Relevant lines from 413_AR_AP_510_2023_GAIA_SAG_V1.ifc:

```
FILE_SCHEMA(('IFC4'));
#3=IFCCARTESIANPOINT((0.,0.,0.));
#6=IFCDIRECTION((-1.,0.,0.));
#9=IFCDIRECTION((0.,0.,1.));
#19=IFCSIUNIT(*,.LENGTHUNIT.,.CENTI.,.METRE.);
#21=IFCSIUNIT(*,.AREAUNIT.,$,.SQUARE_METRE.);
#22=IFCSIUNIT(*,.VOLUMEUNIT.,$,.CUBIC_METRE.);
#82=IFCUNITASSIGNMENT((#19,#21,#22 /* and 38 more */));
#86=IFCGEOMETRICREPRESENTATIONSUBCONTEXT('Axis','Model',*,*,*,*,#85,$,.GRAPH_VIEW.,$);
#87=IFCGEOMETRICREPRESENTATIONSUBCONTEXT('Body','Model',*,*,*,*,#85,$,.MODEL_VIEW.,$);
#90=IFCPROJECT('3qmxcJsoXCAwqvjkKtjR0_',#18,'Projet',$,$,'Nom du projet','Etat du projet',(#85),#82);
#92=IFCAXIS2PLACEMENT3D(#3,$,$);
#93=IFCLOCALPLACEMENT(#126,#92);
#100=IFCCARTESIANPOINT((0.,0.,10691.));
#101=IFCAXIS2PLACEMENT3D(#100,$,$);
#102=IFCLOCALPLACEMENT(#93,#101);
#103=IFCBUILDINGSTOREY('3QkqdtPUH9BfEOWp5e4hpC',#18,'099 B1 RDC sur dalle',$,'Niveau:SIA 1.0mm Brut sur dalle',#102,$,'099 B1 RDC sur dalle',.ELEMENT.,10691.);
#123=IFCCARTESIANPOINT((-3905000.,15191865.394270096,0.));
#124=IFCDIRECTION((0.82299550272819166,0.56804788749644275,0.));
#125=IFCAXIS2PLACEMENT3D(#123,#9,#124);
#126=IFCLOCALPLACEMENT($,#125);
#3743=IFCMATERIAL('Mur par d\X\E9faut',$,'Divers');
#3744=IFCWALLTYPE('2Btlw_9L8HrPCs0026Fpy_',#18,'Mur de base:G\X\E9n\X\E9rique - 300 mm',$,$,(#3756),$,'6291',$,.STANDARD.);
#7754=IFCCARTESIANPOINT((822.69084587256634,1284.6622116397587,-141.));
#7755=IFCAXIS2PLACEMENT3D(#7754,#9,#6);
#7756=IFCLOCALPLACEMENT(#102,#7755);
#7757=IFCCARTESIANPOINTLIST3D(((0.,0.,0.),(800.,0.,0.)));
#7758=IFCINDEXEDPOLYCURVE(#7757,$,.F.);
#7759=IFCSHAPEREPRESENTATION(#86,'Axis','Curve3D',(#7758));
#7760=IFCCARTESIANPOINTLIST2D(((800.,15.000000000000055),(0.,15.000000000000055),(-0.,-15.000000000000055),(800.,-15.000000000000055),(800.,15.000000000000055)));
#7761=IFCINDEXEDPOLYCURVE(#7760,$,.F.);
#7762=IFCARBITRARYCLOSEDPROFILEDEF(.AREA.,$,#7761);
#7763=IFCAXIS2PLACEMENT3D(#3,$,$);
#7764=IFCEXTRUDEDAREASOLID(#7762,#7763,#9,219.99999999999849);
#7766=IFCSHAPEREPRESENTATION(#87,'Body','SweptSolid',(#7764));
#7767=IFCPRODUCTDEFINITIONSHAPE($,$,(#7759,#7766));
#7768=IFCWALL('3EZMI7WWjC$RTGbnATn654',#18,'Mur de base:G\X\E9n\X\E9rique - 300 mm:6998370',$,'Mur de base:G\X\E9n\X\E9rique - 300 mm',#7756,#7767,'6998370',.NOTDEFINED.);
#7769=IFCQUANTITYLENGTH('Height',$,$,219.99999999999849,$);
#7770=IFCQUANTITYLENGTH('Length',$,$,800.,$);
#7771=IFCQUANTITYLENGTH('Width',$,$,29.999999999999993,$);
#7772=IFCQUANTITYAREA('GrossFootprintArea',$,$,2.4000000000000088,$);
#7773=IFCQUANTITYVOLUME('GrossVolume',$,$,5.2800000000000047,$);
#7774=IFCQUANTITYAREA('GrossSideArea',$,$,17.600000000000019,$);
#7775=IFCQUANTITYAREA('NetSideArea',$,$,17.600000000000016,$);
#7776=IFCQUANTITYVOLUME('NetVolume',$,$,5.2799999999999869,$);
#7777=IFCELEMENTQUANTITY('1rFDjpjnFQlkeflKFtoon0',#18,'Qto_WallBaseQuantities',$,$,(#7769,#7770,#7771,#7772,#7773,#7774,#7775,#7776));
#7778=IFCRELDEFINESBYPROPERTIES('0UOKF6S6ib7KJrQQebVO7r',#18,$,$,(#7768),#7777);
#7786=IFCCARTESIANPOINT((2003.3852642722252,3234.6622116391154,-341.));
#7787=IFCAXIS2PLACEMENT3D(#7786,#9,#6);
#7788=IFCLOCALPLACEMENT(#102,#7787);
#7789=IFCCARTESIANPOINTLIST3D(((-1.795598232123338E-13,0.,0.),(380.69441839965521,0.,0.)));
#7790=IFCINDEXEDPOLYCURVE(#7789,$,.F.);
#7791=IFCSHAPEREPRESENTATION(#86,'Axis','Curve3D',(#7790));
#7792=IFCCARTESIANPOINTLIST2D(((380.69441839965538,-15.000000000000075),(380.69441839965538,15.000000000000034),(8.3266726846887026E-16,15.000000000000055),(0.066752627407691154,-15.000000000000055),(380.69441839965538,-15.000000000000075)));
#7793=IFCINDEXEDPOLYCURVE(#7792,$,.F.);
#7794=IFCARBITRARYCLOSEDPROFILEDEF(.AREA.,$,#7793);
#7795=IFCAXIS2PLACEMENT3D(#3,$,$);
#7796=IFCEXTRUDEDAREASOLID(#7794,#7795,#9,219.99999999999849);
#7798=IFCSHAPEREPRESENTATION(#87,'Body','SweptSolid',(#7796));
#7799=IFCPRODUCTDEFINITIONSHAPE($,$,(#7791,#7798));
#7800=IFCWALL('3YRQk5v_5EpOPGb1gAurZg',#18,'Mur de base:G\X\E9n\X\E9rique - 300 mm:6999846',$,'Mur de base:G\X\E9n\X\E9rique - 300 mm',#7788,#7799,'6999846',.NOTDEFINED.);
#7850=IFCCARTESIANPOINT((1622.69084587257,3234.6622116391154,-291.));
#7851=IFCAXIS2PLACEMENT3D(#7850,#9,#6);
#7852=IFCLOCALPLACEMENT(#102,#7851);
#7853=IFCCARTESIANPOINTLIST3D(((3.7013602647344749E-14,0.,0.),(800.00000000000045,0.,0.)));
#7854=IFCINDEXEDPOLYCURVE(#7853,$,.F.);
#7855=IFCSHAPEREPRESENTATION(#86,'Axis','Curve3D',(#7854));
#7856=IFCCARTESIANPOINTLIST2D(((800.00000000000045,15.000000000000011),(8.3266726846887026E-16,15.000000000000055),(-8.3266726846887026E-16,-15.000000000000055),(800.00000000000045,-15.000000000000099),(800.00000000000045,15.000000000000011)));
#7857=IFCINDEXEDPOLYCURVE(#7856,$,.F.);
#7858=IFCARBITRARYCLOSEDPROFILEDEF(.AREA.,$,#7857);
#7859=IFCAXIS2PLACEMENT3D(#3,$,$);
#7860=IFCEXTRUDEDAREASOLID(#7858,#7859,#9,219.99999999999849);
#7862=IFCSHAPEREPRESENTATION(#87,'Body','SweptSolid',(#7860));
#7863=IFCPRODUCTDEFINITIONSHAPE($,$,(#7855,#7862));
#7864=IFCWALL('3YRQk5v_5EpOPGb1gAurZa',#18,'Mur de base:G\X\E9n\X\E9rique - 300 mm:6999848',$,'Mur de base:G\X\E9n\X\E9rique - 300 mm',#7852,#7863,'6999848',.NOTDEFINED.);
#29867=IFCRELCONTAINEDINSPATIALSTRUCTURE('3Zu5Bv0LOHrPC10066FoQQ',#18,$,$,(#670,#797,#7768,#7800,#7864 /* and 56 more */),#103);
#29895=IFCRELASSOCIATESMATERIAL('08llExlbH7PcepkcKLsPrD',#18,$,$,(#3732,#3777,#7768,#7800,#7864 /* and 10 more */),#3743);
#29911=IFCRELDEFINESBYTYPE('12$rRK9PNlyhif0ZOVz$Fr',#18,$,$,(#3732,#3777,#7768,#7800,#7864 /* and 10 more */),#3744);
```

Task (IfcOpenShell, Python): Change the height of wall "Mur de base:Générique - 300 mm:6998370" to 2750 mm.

```python
import ifcopenshell
import ifcopenshell.api.pset
import ifcopenshell.geom
import ifcopenshell.util.element
import ifcopenshell.util.representation
import ifcopenshell.util.shape
import ifcopenshell.util.unit

model = ifcopenshell.open("413_AR_AP_510_2023_GAIA_SAG_V1.ifc")
unit_scale = ifcopenshell.util.unit.calculate_unit_scale(model)
area_scale = ifcopenshell.util.unit.calculate_unit_scale(model, "AREAUNIT")
volume_scale = ifcopenshell.util.unit.calculate_unit_scale(model, "VOLUMEUNIT")
settings = ifcopenshell.geom.settings()


def volume(element):
    """Net volume in cubic metres, openings subtracted."""
    shape = ifcopenshell.geom.create_shape(settings, element)
    return ifcopenshell.util.shape.get_volume(shape.geometry)


wall = model.by_guid("3EZMI7WWjC$RTGbnATn654")
before = volume(wall)

body = ifcopenshell.util.representation.get_representation(wall, "Model", "Body")
solid = body.Items[0]
old_height = solid.Depth
solid.Depth = 2.75 / unit_scale
after = volume(wall)
thickness = 0.3  # wall thickness in metres

# Update the stored height, areas and volumes.
qto = model.by_id(ifcopenshell.util.element.get_pset(wall, "Qto_WallBaseQuantities", should_inherit=False)["id"])
ifcopenshell.api.pset.edit_qto(model, qto=qto, properties={
    "Height": solid.Depth,
    "GrossVolume": ifcopenshell.util.element.get_pset(wall, "Qto_WallBaseQuantities", "GrossVolume") * solid.Depth / old_height,
    "GrossSideArea": ifcopenshell.util.element.get_pset(wall, "Qto_WallBaseQuantities", "GrossSideArea") * solid.Depth / old_height,
    "NetSideArea": after / thickness / area_scale,
    "NetVolume": after / volume_scale,
})

print(f"height {old_height:g} -> {solid.Depth:g}, volume {before:.3f} -> {after:.3f} m3")

model.write("413_AR_AP_510_2023_GAIA_SAG_V1_updated.ifc")
```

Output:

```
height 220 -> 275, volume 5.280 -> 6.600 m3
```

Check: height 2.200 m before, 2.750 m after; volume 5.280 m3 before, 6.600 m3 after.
